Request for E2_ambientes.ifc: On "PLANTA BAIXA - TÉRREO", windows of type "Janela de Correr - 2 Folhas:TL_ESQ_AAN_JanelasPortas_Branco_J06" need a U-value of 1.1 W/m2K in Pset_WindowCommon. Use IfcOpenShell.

First a look at what the model holds.

```python
import ifcopenshell
import ifcopenshell.util.element

model = ifcopenshell.open("E2_ambientes.ifc")
print(model.schema)
storey = next(s for s in model.by_type("IfcBuildingStorey") if s.Name == "PLANTA BAIXA - TÉRREO")
windows = [e for e in ifcopenshell.util.element.get_decomposition(storey) if e.is_a("IfcWindow")]
seen = {}
for e in windows:
    element_type = ifcopenshell.util.element.get_type(e)
    key = (element_type.Name if element_type != e and element_type else None, ifcopenshell.util.element.get_pset(e, "Pset_WindowCommon", "ThermalTransmittance"))
    seen[key] = seen.get(key, 0) + 1
for (name, value), count in sorted(seen.items(), key=str):
    print(count, "x", name, "|", value)
```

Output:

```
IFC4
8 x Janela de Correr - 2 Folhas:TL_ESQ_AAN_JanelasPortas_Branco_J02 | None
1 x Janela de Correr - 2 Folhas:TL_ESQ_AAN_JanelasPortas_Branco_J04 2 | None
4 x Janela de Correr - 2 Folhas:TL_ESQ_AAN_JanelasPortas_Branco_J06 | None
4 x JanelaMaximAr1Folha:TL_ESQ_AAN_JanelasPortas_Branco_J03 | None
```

```python
import ifcopenshell
import ifcopenshell.api.pset
import ifcopenshell.util.element

model = ifcopenshell.open("E2_ambientes.ifc")

storey = next(s for s in model.by_type("IfcBuildingStorey") if s.Name == "PLANTA BAIXA - TÉRREO")
windows = [e for e in ifcopenshell.util.element.get_decomposition(storey) if e.is_a("IfcWindow")]

count = 0
for e in windows:
    element_type = ifcopenshell.util.element.get_type(e)
    if element_type in (None, e) or element_type.Name != "Janela de Correr - 2 Folhas:TL_ESQ_AAN_JanelasPortas_Branco_J06":
        continue
    # add_pset returns the element's existing set when there is one.
    pset = ifcopenshell.api.pset.add_pset(model, product=e, name="Pset_WindowCommon")
    ifcopenshell.api.pset.edit_pset(model, pset=pset, properties={"ThermalTransmittance": 1.1})
    count += 1

print(count, "windows updated")

model.write("E2_ambientes_updated.ifc")
```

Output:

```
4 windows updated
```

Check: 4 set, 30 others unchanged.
